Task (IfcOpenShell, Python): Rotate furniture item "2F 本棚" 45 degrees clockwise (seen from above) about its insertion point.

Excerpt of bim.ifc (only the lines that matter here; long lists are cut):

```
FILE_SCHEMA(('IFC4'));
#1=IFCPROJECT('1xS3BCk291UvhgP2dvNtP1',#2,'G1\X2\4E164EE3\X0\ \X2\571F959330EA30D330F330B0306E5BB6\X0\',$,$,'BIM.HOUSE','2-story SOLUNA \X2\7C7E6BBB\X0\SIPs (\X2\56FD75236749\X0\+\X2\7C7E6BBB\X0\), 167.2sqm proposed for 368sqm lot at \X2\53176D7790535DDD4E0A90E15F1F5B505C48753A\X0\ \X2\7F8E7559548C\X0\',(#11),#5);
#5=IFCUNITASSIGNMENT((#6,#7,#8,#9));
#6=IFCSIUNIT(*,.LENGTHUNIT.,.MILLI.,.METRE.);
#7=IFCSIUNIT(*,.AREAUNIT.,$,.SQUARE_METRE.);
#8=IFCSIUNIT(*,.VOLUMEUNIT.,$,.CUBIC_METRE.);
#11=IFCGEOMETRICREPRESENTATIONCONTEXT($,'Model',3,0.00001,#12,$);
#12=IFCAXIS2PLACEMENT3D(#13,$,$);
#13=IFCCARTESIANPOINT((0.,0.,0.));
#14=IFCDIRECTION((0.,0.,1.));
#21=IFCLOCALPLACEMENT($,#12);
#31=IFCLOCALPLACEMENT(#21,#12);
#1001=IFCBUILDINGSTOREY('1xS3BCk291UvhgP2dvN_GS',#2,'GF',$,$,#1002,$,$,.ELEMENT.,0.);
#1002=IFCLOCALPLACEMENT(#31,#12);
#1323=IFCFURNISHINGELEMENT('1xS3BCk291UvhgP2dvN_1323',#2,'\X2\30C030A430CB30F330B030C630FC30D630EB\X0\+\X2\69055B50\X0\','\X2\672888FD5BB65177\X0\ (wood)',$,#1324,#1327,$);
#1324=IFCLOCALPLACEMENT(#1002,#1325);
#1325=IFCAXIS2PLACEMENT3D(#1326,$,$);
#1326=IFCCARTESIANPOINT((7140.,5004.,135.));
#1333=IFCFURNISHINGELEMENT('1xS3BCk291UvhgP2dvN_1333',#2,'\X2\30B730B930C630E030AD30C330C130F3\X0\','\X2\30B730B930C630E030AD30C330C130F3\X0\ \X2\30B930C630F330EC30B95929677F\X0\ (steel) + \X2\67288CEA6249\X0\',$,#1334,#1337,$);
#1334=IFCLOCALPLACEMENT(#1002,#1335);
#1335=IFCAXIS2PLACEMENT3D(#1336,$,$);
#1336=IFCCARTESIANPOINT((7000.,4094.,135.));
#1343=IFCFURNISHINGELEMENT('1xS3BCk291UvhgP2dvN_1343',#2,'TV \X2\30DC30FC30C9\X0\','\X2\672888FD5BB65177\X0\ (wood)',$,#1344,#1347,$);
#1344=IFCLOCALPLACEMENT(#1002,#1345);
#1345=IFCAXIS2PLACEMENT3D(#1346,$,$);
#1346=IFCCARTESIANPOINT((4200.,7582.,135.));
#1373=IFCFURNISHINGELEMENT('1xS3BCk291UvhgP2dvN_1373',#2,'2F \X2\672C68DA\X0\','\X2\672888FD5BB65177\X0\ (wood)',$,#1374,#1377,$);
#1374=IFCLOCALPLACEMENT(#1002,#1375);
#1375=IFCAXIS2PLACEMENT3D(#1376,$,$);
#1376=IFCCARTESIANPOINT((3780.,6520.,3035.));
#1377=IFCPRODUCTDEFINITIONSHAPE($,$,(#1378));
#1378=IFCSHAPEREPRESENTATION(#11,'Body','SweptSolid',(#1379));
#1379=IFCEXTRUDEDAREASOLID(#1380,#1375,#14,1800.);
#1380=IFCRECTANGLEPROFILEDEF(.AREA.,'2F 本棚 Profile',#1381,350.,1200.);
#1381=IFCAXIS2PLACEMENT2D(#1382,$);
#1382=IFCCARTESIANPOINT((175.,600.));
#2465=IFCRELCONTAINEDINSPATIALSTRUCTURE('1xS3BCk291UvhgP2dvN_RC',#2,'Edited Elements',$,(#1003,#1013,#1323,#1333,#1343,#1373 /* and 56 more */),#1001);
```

```python
import ifcopenshell
import ifcopenshell.api.geometry
import ifcopenshell.util.placement

model = ifcopenshell.open("bim.ifc")

item = model.by_guid("1xS3BCk291UvhgP2dvN_1373")
matrix = ifcopenshell.util.placement.get_local_placement(item.ObjectPlacement)
matrix = matrix @ ifcopenshell.util.placement.rotation(-45, "Z")
ifcopenshell.api.geometry.edit_object_placement(model, product=item, matrix=matrix, is_si=False)

print(ifcopenshell.util.placement.get_local_placement(item.ObjectPlacement).round(3) + 0.0)

model.write("bim_updated.ifc")
```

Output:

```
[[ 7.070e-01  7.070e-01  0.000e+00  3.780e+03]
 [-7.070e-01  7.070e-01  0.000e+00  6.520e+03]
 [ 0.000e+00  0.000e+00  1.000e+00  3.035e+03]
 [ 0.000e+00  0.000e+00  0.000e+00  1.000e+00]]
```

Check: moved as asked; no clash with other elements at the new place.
